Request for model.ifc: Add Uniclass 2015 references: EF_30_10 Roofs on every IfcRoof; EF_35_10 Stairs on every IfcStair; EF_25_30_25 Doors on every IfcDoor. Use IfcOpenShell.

First a look at what the model holds.

```python
import ifcopenshell

model = ifcopenshell.open("model.ifc")
print(model.schema)
print("classifications:", [c.Name for c in model.by_type("IfcClassification")])
for ifc_class in ("IfcDoor", "IfcRoof", "IfcStair", "IfcWall", "IfcWindow"):
    print(ifc_class, len(model.by_type(ifc_class)))
```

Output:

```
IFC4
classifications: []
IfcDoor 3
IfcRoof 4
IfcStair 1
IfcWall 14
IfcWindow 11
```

```python
import ifcopenshell
import ifcopenshell.api.classification

model = ifcopenshell.open("model.ifc")

system = ifcopenshell.api.classification.add_classification(model, classification="Uniclass 2015")

codes = {
    "IfcRoof": ("EF_30_10", "Roofs"),
    "IfcStair": ("EF_35_10", "Stairs"),
    "IfcDoor": ("EF_25_30_25", "Doors"),
}
for ifc_class, (code, name) in codes.items():
    products = model.by_type(ifc_class)
    ifcopenshell.api.classification.add_reference(
        model, products=products, classification=system, identification=code, name=name
    )
    print(code, len(products))

model.write("model_rev.ifc")
```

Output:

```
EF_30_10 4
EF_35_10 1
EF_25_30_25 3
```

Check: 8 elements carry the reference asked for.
